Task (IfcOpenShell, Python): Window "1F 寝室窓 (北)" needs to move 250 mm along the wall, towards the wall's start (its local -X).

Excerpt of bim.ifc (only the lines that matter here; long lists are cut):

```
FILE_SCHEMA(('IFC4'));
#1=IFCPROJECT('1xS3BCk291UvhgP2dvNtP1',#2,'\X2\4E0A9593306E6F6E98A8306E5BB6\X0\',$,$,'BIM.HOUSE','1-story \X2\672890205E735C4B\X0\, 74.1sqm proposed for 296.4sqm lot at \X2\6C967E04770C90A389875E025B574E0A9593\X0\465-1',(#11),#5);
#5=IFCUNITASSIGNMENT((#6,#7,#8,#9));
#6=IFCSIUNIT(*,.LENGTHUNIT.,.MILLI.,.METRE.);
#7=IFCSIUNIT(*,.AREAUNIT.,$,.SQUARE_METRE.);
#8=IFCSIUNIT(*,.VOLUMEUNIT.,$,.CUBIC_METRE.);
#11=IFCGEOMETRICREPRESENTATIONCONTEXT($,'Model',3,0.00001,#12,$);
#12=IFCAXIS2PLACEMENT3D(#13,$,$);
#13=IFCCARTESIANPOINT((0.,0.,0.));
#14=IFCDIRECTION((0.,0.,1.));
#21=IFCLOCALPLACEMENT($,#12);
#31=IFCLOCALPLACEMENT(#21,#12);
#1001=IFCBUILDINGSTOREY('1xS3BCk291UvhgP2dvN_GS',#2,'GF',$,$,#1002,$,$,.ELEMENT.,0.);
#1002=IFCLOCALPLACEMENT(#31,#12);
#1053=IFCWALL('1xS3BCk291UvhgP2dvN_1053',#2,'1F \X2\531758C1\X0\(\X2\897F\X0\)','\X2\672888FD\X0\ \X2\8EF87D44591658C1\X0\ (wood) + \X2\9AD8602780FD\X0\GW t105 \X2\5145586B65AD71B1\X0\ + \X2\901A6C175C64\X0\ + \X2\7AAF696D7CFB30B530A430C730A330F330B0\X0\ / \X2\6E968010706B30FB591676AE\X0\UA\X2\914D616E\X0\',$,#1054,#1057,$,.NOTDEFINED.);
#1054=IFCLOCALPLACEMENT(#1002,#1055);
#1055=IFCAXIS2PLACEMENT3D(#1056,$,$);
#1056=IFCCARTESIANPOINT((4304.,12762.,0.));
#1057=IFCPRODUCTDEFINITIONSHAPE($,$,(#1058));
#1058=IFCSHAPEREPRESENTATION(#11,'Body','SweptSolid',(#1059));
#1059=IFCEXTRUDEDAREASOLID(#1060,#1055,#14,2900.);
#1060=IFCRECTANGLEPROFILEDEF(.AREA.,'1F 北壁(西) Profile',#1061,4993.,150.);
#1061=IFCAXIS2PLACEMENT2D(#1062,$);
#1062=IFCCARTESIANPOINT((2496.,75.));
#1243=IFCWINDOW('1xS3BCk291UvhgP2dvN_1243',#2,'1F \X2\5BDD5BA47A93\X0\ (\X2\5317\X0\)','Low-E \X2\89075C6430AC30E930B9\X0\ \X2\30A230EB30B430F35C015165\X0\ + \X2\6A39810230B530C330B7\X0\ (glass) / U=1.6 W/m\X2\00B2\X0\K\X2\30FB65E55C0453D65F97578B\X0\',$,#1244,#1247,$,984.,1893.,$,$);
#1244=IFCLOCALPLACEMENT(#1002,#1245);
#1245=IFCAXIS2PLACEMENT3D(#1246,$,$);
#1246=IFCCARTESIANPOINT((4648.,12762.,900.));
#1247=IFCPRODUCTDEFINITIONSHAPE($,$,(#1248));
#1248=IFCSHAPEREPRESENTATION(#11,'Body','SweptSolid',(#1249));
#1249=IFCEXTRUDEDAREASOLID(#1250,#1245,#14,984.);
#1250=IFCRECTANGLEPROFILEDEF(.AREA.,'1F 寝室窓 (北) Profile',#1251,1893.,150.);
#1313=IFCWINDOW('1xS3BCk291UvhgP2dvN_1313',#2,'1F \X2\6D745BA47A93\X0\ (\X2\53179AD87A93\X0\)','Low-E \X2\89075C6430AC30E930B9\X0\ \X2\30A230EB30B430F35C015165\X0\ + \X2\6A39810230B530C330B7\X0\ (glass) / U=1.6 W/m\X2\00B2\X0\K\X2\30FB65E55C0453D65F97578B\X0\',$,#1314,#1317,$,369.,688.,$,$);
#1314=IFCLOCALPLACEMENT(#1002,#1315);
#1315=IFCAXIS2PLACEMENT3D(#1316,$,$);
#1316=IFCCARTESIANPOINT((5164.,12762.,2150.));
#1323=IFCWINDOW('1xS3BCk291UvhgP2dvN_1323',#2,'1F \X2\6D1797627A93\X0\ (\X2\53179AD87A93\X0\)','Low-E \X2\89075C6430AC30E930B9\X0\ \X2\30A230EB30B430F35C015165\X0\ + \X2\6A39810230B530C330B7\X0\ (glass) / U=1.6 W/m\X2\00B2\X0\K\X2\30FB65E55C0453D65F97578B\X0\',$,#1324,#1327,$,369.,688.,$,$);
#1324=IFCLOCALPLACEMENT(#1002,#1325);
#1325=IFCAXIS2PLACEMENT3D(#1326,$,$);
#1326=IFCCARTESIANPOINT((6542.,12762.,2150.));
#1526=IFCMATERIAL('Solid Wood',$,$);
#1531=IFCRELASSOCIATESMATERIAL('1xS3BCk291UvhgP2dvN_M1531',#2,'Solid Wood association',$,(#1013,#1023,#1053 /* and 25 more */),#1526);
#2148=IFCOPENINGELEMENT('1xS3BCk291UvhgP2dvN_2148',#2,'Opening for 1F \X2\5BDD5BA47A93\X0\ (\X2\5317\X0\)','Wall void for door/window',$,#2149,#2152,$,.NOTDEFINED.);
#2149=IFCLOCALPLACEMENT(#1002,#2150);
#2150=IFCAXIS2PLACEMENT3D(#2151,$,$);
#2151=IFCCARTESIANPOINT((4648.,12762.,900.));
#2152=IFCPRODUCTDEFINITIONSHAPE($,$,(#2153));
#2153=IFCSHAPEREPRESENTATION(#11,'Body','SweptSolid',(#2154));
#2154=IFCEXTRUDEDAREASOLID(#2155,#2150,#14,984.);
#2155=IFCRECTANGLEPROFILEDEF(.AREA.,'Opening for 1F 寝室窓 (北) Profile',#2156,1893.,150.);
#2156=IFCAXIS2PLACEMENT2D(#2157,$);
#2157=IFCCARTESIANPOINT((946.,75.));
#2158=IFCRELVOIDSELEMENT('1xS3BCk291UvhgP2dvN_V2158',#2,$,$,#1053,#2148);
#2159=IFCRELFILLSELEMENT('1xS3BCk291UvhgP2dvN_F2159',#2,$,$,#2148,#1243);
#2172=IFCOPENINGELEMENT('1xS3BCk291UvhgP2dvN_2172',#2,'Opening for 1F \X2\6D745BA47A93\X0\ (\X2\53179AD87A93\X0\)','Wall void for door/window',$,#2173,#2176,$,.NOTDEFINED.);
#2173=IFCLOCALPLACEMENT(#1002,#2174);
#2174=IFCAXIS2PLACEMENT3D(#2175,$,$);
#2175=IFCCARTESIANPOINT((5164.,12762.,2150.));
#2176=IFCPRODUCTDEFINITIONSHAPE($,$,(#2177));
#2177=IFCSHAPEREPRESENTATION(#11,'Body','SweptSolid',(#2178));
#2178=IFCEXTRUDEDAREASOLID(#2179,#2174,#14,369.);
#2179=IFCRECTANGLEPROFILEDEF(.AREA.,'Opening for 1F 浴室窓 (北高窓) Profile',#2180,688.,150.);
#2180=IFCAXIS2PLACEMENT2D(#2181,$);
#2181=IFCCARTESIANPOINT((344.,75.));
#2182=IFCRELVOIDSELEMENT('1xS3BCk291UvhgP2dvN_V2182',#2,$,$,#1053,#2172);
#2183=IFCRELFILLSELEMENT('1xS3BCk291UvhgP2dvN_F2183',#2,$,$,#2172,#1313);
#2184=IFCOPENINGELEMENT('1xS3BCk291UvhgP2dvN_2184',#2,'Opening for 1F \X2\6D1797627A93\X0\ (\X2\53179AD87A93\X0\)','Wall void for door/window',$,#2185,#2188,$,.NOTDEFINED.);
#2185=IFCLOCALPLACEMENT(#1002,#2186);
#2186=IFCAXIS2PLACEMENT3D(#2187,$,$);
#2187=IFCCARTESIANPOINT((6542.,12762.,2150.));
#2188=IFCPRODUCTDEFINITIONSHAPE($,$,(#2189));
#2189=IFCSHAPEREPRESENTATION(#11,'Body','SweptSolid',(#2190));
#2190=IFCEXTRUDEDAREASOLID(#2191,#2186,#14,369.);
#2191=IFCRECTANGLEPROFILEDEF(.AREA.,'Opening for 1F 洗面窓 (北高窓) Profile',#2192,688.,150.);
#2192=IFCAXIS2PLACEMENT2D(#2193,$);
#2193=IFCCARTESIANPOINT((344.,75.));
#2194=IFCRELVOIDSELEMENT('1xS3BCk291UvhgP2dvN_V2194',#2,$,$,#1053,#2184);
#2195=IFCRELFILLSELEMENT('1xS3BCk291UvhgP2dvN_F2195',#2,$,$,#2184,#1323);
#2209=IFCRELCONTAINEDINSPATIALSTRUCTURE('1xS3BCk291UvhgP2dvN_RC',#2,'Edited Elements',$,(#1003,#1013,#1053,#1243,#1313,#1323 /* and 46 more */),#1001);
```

```python
import ifcopenshell
import ifcopenshell.api.geometry
import ifcopenshell.util.placement

model = ifcopenshell.open("bim.ifc")

window = model.by_guid("1xS3BCk291UvhgP2dvN_1243")
opening = window.FillsVoids[0].RelatingOpeningElement
wall = opening.VoidsElements[0].RelatingBuildingElement

wall_matrix = ifcopenshell.util.placement.get_local_placement(wall.ObjectPlacement)
shift = wall_matrix[:3, 0] * -250.0
before = ifcopenshell.util.placement.get_local_placement(window.ObjectPlacement)[:3, 3].copy()

# The window is not placed relative to its opening, so move both.
for product in (opening, window):
    matrix = ifcopenshell.util.placement.get_local_placement(product.ObjectPlacement)
    matrix[:3, 3] += shift
    ifcopenshell.api.geometry.edit_object_placement(model, product=product, matrix=matrix, is_si=False)

after = ifcopenshell.util.placement.get_local_placement(window.ObjectPlacement)[:3, 3]
print("window moved by", (after - before).round(3) + 0.0)

model.write("bim-out.ifc")
```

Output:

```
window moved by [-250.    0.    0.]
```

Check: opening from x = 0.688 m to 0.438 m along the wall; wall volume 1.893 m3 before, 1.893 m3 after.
